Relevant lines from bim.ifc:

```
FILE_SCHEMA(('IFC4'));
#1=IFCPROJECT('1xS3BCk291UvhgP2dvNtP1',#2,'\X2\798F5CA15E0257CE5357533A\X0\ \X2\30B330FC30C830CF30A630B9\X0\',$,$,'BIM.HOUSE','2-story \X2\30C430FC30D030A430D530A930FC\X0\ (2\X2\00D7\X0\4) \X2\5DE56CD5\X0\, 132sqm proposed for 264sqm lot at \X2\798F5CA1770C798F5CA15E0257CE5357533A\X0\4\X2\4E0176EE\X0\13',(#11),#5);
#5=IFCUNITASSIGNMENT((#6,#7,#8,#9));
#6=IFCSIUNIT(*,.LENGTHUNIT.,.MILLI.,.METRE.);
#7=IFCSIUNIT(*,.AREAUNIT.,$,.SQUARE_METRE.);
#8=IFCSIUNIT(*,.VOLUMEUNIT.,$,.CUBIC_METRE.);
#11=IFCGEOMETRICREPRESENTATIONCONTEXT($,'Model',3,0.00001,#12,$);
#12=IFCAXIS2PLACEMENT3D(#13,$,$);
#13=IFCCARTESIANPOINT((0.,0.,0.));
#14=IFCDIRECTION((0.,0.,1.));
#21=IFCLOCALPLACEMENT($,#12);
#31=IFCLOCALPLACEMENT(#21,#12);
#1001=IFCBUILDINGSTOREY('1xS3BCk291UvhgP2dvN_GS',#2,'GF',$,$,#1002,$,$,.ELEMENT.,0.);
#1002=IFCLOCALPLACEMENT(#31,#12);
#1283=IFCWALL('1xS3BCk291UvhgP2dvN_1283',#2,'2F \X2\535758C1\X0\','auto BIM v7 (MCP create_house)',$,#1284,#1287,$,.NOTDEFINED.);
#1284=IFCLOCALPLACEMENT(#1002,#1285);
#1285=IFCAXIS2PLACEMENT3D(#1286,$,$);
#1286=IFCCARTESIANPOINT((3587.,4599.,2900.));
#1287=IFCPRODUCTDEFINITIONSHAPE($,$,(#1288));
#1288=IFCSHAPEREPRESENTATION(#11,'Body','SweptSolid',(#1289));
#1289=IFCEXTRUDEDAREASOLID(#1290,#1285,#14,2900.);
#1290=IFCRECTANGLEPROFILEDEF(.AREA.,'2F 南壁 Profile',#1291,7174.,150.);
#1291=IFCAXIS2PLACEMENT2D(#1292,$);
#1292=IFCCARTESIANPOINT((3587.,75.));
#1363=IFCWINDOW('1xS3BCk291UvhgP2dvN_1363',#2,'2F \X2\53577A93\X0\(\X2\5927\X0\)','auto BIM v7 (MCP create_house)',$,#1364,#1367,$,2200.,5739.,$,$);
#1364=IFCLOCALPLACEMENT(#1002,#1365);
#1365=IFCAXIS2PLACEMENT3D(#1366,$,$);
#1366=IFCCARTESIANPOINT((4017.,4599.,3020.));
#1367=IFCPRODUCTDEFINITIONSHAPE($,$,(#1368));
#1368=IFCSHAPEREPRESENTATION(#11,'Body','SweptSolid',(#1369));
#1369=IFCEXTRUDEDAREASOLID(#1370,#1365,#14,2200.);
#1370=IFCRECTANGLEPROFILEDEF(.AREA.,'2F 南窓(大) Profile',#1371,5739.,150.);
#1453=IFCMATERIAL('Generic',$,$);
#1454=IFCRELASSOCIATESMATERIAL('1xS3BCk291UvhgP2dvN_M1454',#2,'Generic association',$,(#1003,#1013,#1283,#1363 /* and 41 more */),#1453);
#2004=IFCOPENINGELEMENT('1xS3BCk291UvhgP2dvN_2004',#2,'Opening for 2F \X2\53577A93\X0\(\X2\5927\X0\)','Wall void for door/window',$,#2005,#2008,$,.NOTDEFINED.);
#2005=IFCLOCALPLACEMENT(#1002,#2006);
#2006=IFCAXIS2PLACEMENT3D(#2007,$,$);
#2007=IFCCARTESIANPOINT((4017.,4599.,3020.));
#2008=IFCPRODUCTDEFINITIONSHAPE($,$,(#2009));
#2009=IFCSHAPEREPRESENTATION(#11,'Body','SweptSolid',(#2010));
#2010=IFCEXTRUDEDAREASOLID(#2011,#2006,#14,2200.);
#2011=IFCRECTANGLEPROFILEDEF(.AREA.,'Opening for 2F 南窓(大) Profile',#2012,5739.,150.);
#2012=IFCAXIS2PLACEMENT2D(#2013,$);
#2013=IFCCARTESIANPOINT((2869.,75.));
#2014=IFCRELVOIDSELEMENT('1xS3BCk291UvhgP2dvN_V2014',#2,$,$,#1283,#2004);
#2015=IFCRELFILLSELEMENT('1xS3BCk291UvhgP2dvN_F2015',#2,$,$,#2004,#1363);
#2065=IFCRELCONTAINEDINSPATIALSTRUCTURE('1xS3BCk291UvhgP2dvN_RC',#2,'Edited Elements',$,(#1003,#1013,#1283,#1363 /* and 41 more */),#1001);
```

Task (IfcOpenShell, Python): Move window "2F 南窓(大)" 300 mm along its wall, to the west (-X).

```python
import ifcopenshell
import ifcopenshell.api.geometry
import ifcopenshell.util.placement
import ifcopenshell.util.unit

model = ifcopenshell.open("bim.ifc")
unit_scale = ifcopenshell.util.unit.calculate_unit_scale(model)

window = model.by_guid("1xS3BCk291UvhgP2dvN_1363")
opening = window.FillsVoids[0].RelatingOpeningElement
wall = opening.VoidsElements[0].RelatingBuildingElement

wall_matrix = ifcopenshell.util.placement.get_local_placement(wall.ObjectPlacement)
shift = wall_matrix[:3, 0] * -0.3 / unit_scale
before = ifcopenshell.util.placement.get_local_placement(window.ObjectPlacement)[:3, 3].copy()

# The window is not placed relative to its opening, so move both.
for product in (opening, window):
    matrix = ifcopenshell.util.placement.get_local_placement(product.ObjectPlacement)
    matrix[:3, 3] += shift
    ifcopenshell.api.geometry.edit_object_placement(model, product=product, matrix=matrix, is_si=False)

after = ifcopenshell.util.placement.get_local_placement(window.ObjectPlacement)[:3, 3]
print("window moved by", (after - before).round(3) + 0.0)

model.write("bim_rev.ifc")
```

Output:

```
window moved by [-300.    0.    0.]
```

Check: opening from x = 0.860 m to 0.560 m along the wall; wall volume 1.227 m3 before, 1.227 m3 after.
